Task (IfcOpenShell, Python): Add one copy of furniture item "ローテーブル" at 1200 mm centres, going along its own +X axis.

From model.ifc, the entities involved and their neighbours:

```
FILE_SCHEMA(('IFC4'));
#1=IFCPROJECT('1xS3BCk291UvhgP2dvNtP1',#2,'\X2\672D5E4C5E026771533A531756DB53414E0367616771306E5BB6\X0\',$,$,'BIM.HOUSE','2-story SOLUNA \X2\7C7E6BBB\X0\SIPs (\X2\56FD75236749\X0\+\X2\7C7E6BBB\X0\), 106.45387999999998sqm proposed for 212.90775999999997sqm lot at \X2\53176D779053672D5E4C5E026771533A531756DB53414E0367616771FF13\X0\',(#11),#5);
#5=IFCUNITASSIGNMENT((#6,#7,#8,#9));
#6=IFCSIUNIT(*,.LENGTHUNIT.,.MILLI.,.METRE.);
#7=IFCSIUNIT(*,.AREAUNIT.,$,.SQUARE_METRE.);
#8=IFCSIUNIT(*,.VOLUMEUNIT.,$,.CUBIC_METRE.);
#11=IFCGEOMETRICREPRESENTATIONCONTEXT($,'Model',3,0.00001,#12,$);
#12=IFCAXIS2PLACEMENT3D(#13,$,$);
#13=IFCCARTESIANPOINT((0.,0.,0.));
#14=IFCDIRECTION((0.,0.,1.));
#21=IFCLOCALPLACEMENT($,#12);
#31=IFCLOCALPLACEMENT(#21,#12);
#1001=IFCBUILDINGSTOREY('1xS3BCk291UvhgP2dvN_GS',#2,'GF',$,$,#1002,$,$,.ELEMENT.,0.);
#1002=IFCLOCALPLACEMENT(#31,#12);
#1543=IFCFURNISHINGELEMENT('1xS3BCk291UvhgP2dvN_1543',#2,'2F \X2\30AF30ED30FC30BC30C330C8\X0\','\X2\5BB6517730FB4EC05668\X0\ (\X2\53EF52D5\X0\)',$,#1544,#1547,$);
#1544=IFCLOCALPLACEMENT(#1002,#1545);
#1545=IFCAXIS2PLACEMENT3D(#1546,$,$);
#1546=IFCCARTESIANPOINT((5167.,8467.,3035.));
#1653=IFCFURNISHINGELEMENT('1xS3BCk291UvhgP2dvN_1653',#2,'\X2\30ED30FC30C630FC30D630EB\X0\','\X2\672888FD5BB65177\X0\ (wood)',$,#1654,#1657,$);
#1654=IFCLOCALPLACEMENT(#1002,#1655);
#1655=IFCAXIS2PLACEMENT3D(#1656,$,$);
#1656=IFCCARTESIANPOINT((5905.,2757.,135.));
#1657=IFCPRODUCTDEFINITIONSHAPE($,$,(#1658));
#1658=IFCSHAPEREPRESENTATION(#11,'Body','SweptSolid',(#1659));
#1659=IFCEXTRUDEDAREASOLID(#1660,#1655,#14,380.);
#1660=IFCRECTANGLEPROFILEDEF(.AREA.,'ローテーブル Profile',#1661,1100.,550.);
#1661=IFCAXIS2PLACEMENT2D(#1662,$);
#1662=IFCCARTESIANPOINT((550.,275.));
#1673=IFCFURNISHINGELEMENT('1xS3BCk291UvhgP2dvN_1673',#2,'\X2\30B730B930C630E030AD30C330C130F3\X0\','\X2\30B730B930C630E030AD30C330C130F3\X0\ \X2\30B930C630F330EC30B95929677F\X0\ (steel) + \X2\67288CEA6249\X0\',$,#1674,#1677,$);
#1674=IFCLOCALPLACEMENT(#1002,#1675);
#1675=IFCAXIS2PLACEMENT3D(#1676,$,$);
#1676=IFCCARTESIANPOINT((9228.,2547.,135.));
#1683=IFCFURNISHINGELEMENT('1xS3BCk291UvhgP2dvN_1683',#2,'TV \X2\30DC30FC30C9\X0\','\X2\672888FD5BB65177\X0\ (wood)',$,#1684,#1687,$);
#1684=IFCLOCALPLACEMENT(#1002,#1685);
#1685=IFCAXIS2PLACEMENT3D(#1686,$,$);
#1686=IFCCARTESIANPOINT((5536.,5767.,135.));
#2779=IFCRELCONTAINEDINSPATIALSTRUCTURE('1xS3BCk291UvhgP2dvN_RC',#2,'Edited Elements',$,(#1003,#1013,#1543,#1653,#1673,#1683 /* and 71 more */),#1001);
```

```python
import ifcopenshell
import ifcopenshell.api.geometry
import ifcopenshell.api.root
import ifcopenshell.util.element
import ifcopenshell.util.placement
import ifcopenshell.util.unit

model = ifcopenshell.open("model.ifc")
unit_scale = ifcopenshell.util.unit.calculate_unit_scale(model)


def reuse_history(source, copy):
    """copy_class also copies each property set's owner history, people and application; keep the originals."""
    for rel in copy.IsDefinedBy:
        if rel.is_a("IfcRelDefinesByProperties") and (history := rel.RelatingPropertyDefinition.OwnerHistory):
            rel.RelatingPropertyDefinition.OwnerHistory = source.OwnerHistory
            ifcopenshell.util.element.remove_deep2(model, history)


source = model.by_id(1653)
base = ifcopenshell.util.placement.get_local_placement(source.ObjectPlacement)
step = base[:3, 0] * 1.2 / unit_scale

for i in range(1, 2):
    copy = ifcopenshell.api.root.copy_class(model, product=source)
    copy.Representation = ifcopenshell.util.element.copy_deep(
        model, source.Representation, exclude=["IfcGeometricRepresentationContext", "IfcRepresentationMap"]
    )
    reuse_history(source, copy)
    matrix = base.copy()
    matrix[:3, 3] += i * step
    print("added at", matrix[:3, 3].round(3) + 0.0)
    ifcopenshell.api.geometry.edit_object_placement(model, product=copy, matrix=matrix, is_si=False)

model.write("model_updated.ifc")
```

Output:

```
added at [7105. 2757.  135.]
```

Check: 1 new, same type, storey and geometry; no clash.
